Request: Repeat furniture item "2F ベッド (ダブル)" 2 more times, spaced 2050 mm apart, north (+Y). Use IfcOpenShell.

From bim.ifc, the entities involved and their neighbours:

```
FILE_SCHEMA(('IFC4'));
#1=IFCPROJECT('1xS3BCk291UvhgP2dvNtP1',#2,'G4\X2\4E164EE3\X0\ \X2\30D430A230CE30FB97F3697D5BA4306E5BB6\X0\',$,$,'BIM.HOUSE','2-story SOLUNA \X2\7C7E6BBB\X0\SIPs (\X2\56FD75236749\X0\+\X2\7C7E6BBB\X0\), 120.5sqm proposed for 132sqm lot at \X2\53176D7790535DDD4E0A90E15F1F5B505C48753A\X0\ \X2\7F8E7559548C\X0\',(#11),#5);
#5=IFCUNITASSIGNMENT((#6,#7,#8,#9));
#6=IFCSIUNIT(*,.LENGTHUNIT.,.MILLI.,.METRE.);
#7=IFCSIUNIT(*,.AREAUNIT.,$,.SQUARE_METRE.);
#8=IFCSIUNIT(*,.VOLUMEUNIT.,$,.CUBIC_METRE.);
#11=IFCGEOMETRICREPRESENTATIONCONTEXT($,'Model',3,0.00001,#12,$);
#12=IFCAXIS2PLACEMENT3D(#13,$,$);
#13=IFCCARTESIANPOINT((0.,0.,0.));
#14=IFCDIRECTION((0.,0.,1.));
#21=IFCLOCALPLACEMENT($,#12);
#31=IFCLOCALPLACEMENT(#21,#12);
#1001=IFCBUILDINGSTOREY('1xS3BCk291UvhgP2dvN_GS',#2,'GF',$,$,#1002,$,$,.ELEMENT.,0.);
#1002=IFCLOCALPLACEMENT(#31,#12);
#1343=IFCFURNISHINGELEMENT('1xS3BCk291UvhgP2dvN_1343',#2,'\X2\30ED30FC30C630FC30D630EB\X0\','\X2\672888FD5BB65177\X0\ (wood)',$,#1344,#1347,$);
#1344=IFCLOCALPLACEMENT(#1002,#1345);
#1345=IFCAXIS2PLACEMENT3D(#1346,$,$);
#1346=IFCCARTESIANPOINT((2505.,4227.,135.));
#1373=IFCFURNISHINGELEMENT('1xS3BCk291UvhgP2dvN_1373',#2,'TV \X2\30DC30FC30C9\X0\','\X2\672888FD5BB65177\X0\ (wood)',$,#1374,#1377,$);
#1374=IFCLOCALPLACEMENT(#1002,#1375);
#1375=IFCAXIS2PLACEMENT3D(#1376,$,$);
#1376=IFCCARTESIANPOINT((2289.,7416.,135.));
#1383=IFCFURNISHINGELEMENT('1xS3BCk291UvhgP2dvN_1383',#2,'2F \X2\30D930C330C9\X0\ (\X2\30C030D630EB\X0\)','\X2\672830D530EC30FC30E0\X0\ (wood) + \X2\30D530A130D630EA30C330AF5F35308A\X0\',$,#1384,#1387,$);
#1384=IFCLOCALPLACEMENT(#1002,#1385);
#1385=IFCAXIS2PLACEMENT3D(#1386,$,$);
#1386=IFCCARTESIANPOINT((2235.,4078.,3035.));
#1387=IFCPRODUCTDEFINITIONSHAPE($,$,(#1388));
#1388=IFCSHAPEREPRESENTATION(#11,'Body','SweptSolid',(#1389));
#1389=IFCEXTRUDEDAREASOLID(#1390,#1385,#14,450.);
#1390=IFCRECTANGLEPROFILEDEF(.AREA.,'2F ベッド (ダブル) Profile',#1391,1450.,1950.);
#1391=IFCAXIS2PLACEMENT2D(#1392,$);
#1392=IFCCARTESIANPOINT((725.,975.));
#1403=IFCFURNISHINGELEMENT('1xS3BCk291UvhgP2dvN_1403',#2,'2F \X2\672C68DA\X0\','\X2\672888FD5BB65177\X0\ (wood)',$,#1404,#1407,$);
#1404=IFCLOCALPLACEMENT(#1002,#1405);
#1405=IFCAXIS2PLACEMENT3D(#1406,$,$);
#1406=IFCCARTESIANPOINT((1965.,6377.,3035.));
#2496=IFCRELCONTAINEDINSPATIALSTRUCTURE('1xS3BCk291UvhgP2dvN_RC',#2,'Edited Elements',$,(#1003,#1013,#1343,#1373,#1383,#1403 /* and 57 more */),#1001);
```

```python
import numpy as np
import ifcopenshell
import ifcopenshell.api.geometry
import ifcopenshell.api.root
import ifcopenshell.util.element
import ifcopenshell.util.placement
import ifcopenshell.util.unit

model = ifcopenshell.open("bim.ifc")
unit_scale = ifcopenshell.util.unit.calculate_unit_scale(model)


def reuse_history(source, copy):
    """copy_class also copies each property set's owner history, people and application; keep the originals."""
    for rel in copy.IsDefinedBy:
        if rel.is_a("IfcRelDefinesByProperties") and (history := rel.RelatingPropertyDefinition.OwnerHistory):
            rel.RelatingPropertyDefinition.OwnerHistory = source.OwnerHistory
            ifcopenshell.util.element.remove_deep2(model, history)


source = model.by_id(1383)
base = ifcopenshell.util.placement.get_local_placement(source.ObjectPlacement)
step = np.array([0.0, 1.0, 0.0]) * 2.05 / unit_scale

for i in range(1, 3):
    copy = ifcopenshell.api.root.copy_class(model, product=source)
    copy.Representation = ifcopenshell.util.element.copy_deep(
        model, source.Representation, exclude=["IfcGeometricRepresentationContext", "IfcRepresentationMap"]
    )
    reuse_history(source, copy)
    matrix = base.copy()
    matrix[:3, 3] += i * step
    print("added at", matrix[:3, 3].round(3) + 0.0)
    ifcopenshell.api.geometry.edit_object_placement(model, product=copy, matrix=matrix, is_si=False)

model.write("bim_rev.ifc")
```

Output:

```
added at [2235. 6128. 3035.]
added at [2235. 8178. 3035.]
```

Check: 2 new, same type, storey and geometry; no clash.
